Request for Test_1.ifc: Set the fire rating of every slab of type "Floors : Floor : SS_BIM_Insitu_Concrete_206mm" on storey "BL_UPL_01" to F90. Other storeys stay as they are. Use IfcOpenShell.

First a look at what the model holds.

```python
import ifcopenshell
import ifcopenshell.util.element

model = ifcopenshell.open("Test_1.ifc")
print(model.schema)
storey = next(s for s in model.by_type("IfcBuildingStorey") if s.Name == "BL_UPL_01")
slabs = [e for e in ifcopenshell.util.element.get_decomposition(storey) if e.is_a("IfcSlab")]
seen = {}
for e in slabs:
    element_type = ifcopenshell.util.element.get_type(e)
    key = (element_type.Name if element_type != e and element_type else None, ifcopenshell.util.element.get_pset(e, "Pset_SlabCommon", "FireRating"))
    seen[key] = seen.get(key, 0) + 1
for (name, value), count in sorted(seen.items(), key=str):
    print(count, "x", name, "|", value)
```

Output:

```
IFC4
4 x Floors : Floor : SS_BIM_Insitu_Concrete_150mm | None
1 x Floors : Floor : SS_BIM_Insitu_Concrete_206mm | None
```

```python
import ifcopenshell
import ifcopenshell.api.pset
import ifcopenshell.util.element

model = ifcopenshell.open("Test_1.ifc")

storey = next(s for s in model.by_type("IfcBuildingStorey") if s.Name == "BL_UPL_01")
slabs = [e for e in ifcopenshell.util.element.get_decomposition(storey) if e.is_a("IfcSlab")]

count = 0
for e in slabs:
    element_type = ifcopenshell.util.element.get_type(e)
    if element_type in (None, e) or element_type.Name != "Floors : Floor : SS_BIM_Insitu_Concrete_206mm":
        continue
    # add_pset returns the element's existing set when there is one.
    pset = ifcopenshell.api.pset.add_pset(model, product=e, name="Pset_SlabCommon")
    ifcopenshell.api.pset.edit_pset(model, pset=pset, properties={"FireRating": "F90"})
    count += 1

print(count, "slabs updated")

model.write("Test_1_edited.ifc")
```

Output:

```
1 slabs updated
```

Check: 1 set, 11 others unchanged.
